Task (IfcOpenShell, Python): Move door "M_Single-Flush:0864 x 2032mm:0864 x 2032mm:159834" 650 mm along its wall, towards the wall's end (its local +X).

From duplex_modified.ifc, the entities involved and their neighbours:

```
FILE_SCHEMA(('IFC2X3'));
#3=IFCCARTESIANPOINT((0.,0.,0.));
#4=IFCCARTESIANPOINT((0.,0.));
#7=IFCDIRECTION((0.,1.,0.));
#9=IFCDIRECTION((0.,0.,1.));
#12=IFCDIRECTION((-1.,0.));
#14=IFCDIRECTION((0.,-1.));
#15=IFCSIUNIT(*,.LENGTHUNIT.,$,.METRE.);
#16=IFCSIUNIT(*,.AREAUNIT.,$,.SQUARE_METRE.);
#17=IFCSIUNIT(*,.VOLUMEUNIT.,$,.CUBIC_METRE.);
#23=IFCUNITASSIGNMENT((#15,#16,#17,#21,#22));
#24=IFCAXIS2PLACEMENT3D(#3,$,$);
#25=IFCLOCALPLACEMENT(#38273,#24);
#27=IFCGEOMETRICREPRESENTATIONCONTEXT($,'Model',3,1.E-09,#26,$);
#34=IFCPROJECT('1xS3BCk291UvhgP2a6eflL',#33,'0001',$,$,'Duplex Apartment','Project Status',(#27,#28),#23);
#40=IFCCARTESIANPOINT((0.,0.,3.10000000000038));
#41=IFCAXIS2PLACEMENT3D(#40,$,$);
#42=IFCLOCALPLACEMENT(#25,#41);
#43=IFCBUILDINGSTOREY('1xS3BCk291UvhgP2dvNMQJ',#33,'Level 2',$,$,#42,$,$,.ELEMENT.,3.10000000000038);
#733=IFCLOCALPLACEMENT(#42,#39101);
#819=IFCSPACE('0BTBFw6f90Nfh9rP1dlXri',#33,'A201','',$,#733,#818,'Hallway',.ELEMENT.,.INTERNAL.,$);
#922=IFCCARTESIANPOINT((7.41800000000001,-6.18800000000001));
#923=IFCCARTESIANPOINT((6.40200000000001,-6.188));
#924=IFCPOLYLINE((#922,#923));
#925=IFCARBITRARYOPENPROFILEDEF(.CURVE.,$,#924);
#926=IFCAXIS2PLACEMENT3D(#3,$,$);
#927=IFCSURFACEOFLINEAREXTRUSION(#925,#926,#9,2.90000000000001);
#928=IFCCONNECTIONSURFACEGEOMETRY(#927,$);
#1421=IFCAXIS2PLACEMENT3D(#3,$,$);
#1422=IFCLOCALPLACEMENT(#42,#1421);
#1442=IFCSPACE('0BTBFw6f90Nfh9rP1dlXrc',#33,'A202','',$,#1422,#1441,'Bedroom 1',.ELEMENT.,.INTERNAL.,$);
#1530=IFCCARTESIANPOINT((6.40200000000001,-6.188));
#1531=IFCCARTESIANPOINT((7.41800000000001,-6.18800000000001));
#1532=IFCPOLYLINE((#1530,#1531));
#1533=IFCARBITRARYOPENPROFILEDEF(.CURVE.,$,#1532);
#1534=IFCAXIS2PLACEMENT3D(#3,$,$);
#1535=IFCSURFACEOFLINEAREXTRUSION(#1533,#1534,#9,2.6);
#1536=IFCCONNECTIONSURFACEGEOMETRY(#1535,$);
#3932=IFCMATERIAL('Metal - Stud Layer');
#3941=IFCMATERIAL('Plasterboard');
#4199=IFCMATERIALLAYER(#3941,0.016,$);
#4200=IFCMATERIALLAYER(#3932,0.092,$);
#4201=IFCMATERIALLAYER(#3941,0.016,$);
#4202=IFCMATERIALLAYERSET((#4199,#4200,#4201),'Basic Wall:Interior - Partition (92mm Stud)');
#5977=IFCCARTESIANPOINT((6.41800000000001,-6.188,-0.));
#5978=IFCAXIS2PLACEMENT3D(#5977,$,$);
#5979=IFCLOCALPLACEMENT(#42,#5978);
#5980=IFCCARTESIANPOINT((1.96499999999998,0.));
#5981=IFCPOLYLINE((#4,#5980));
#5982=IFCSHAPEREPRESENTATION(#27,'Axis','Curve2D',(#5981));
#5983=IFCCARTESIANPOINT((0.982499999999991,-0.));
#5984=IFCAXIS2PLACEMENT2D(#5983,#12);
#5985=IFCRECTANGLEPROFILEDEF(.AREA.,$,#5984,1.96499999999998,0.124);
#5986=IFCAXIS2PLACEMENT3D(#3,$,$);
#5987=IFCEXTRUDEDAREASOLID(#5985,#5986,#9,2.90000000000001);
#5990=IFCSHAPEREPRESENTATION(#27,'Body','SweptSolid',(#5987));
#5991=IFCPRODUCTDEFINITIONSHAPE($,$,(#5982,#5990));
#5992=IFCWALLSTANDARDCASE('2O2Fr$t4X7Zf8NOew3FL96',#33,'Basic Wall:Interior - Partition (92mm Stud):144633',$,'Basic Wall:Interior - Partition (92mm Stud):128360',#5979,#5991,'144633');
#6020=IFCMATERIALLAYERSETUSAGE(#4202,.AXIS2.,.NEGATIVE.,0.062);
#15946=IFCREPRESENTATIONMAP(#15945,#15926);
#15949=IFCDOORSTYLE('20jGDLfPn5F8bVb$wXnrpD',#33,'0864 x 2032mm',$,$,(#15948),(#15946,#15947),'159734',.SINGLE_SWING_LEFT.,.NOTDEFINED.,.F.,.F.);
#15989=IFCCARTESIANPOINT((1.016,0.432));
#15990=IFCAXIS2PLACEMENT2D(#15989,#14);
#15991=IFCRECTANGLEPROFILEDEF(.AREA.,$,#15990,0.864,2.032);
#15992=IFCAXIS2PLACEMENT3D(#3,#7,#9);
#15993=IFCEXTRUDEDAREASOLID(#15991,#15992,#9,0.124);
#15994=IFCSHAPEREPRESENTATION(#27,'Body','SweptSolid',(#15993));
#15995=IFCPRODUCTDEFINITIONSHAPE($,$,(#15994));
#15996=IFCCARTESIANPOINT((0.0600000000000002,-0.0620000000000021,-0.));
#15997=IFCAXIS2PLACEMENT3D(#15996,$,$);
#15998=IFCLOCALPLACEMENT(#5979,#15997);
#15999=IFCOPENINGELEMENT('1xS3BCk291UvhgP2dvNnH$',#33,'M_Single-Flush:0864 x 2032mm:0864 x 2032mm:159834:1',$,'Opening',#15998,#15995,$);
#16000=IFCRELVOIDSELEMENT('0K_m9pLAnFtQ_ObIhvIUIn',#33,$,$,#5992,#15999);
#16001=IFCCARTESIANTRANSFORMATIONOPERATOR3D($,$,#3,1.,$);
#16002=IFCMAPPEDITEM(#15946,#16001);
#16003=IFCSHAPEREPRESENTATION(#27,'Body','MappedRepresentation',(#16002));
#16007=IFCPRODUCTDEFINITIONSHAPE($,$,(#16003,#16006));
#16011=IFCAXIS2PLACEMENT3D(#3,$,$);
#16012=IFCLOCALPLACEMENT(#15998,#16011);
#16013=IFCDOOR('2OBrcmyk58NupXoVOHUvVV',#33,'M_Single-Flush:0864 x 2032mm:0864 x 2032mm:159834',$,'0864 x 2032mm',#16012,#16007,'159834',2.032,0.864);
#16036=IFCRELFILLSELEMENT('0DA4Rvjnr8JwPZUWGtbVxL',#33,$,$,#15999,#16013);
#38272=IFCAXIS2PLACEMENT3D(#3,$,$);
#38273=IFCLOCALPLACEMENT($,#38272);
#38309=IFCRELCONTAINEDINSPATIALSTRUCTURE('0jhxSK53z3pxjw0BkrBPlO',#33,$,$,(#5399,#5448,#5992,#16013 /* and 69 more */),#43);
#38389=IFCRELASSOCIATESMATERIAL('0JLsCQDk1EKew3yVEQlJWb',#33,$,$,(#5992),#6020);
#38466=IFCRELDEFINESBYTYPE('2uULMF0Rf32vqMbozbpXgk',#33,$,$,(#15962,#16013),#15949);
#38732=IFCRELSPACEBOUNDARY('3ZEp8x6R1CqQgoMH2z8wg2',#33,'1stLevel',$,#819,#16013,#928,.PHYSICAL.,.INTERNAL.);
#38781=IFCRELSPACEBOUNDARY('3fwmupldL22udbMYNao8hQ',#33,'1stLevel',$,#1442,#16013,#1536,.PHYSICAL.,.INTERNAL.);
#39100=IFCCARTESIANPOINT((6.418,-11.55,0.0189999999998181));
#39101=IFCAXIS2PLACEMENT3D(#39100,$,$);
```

```python
import numpy as np
import ifcopenshell
import ifcopenshell.api.geometry
import ifcopenshell.util.placement
import ifcopenshell.util.unit

model = ifcopenshell.open("duplex_modified.ifc")
unit_scale = ifcopenshell.util.unit.calculate_unit_scale(model)

door = model.by_id(16013)
opening = door.FillsVoids[0].RelatingOpeningElement
wall = opening.VoidsElements[0].RelatingBuildingElement

wall_matrix = ifcopenshell.util.placement.get_local_placement(wall.ObjectPlacement)
shift = wall_matrix[:3, 0] * 0.65 / unit_scale
before = ifcopenshell.util.placement.get_local_placement(door.ObjectPlacement)[:3, 3].copy()

# The door is placed relative to its opening, so it follows when the opening moves.
matrix = ifcopenshell.util.placement.get_local_placement(opening.ObjectPlacement)
matrix[:3, 3] += shift
ifcopenshell.api.geometry.edit_object_placement(
    model, product=opening, matrix=matrix, is_si=False, should_transform_children=True
)

# Space boundary surfaces are stored in each space's coordinates; move them too.
for rel in door.ProvidesBoundaries:
    if not rel.ConnectionGeometry:
        continue
    surface = rel.ConnectionGeometry.SurfaceOnRelatingElement
    space_matrix = ifcopenshell.util.placement.get_local_placement(rel.RelatingSpace.ObjectPlacement)
    point = np.array(surface.Position.Location.Coordinates) + space_matrix[:3, :3].T @ shift
    surface.Position = model.createIfcAxis2Placement3D(
        model.createIfcCartesianPoint(point.tolist()), surface.Position.Axis, surface.Position.RefDirection
    )

after = ifcopenshell.util.placement.get_local_placement(door.ObjectPlacement)[:3, 3]
print("door moved by", (after - before).round(3) + 0.0)

model.write("duplex_modified_edited.ifc")
```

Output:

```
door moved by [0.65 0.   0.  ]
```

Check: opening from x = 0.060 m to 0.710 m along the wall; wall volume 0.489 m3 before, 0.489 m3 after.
